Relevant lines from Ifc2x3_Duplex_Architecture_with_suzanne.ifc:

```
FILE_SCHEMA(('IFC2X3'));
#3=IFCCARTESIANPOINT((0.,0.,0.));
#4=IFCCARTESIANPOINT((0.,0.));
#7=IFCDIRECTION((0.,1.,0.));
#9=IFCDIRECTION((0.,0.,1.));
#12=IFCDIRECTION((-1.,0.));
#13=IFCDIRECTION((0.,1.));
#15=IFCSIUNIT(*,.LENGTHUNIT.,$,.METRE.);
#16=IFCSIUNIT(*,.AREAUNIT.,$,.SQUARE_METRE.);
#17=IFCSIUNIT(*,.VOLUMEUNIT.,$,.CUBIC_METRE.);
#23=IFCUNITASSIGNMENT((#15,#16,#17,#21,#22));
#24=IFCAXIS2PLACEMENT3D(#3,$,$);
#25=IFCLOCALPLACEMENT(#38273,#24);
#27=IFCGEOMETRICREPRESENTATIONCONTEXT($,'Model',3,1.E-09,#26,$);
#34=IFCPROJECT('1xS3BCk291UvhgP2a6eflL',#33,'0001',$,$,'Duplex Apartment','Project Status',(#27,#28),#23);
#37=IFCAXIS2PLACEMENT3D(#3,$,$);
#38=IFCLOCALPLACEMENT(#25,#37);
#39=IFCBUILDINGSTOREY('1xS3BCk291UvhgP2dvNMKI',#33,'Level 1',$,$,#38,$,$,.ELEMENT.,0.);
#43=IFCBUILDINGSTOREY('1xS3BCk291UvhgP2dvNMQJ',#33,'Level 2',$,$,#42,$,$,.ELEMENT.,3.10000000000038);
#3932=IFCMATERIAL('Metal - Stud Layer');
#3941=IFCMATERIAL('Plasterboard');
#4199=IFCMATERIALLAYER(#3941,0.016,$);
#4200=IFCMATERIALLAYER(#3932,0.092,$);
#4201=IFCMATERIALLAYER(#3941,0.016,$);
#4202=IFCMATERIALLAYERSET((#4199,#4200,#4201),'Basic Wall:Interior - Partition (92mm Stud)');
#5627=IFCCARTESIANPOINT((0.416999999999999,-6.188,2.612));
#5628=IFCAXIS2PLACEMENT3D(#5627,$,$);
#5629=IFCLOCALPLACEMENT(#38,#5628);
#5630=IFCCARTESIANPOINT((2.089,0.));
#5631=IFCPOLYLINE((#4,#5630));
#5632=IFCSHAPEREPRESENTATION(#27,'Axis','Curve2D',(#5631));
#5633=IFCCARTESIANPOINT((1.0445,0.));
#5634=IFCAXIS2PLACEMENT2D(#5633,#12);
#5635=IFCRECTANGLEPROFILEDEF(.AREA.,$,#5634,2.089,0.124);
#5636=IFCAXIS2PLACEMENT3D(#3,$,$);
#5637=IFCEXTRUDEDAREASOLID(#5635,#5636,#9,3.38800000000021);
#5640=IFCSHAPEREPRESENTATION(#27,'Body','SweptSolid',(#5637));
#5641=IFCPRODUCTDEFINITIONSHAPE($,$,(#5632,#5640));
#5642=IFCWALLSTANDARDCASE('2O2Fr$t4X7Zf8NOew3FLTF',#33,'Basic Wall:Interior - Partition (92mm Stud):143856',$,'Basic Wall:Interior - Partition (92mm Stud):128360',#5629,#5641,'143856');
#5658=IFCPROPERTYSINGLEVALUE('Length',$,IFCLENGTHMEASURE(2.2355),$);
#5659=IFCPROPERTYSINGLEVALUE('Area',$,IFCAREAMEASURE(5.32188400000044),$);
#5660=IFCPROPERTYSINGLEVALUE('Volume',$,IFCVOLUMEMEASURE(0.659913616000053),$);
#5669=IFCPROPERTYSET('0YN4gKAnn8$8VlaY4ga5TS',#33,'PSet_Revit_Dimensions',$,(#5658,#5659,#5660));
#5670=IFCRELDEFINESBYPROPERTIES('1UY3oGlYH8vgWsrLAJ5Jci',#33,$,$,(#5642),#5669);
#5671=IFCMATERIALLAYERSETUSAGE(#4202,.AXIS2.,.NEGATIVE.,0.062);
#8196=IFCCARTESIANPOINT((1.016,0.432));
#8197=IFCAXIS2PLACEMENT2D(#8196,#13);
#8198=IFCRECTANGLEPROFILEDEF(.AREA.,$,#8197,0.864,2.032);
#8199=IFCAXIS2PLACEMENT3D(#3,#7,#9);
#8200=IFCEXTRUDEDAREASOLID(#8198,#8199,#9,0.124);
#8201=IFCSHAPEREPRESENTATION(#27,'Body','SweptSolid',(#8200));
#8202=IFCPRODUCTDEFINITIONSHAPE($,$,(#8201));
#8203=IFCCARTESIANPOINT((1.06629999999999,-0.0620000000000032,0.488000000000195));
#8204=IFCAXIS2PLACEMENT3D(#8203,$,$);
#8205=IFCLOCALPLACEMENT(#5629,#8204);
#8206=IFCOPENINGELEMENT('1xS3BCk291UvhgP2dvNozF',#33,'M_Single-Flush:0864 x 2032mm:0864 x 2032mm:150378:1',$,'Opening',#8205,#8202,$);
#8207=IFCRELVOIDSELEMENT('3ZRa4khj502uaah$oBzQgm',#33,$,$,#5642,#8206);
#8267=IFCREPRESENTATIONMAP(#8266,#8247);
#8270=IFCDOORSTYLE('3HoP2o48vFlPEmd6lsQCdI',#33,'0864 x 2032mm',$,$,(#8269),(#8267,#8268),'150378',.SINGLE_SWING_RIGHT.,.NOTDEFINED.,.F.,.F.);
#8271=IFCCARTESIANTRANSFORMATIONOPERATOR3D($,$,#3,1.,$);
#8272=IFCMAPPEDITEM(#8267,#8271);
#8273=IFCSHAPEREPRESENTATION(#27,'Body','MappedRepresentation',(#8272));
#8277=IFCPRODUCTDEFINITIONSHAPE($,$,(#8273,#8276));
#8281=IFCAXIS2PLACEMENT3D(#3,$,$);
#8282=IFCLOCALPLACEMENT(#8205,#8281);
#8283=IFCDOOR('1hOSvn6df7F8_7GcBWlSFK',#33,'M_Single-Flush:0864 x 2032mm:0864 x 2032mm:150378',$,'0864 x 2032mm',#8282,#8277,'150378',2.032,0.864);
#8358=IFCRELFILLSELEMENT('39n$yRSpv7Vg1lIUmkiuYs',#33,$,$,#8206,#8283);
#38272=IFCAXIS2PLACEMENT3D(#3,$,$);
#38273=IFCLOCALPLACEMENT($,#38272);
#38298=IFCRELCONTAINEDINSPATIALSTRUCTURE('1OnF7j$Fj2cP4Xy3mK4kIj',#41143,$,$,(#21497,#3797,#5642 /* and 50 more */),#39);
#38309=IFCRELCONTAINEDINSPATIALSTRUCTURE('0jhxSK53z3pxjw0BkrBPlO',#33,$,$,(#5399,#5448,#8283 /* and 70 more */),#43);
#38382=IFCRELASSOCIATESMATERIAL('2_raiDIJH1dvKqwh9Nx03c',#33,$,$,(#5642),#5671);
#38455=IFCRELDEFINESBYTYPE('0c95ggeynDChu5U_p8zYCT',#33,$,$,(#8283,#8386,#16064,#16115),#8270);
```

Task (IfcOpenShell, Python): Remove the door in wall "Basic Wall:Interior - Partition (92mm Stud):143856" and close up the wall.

```python
import ifcopenshell
import ifcopenshell.api.feature
import ifcopenshell.api.pset
import ifcopenshell.api.root
import ifcopenshell.geom
import ifcopenshell.util.element
import ifcopenshell.util.shape
import ifcopenshell.util.unit

model = ifcopenshell.open("Ifc2x3_Duplex_Architecture_with_suzanne.ifc")
area_scale = ifcopenshell.util.unit.calculate_unit_scale(model, "AREAUNIT")
volume_scale = ifcopenshell.util.unit.calculate_unit_scale(model, "VOLUMEUNIT")
settings = ifcopenshell.geom.settings()


def volume(element):
    """Net volume in cubic metres, openings subtracted."""
    shape = ifcopenshell.geom.create_shape(settings, element)
    return ifcopenshell.util.shape.get_volume(shape.geometry)


door = model.by_guid("1hOSvn6df7F8_7GcBWlSFK")
opening = door.FillsVoids[0].RelatingOpeningElement
wall = opening.VoidsElements[0].RelatingBuildingElement
before = volume(wall)

ifcopenshell.api.root.remove_product(model, product=door)
ifcopenshell.api.feature.remove_feature(model, feature=opening)

after = volume(wall)
thickness = 0.124  # wall thickness in metres

# Update the wall's stored quantities.
pset = model.by_id(ifcopenshell.util.element.get_pset(wall, "PSet_Revit_Dimensions", should_inherit=False)["id"])
ifcopenshell.api.pset.edit_pset(model, pset=pset, properties={
    "Area": model.create_entity("IfcAreaMeasure", after / thickness / area_scale),
    "Volume": model.create_entity("IfcVolumeMeasure", after / volume_scale),
})

print(f"wall volume {before:.3f} -> {after:.3f} m3")

model.write("Ifc2x3_Duplex_Architecture_with_suzanne_rev.ifc")
```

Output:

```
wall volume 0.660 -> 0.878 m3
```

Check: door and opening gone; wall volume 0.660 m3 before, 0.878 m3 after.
